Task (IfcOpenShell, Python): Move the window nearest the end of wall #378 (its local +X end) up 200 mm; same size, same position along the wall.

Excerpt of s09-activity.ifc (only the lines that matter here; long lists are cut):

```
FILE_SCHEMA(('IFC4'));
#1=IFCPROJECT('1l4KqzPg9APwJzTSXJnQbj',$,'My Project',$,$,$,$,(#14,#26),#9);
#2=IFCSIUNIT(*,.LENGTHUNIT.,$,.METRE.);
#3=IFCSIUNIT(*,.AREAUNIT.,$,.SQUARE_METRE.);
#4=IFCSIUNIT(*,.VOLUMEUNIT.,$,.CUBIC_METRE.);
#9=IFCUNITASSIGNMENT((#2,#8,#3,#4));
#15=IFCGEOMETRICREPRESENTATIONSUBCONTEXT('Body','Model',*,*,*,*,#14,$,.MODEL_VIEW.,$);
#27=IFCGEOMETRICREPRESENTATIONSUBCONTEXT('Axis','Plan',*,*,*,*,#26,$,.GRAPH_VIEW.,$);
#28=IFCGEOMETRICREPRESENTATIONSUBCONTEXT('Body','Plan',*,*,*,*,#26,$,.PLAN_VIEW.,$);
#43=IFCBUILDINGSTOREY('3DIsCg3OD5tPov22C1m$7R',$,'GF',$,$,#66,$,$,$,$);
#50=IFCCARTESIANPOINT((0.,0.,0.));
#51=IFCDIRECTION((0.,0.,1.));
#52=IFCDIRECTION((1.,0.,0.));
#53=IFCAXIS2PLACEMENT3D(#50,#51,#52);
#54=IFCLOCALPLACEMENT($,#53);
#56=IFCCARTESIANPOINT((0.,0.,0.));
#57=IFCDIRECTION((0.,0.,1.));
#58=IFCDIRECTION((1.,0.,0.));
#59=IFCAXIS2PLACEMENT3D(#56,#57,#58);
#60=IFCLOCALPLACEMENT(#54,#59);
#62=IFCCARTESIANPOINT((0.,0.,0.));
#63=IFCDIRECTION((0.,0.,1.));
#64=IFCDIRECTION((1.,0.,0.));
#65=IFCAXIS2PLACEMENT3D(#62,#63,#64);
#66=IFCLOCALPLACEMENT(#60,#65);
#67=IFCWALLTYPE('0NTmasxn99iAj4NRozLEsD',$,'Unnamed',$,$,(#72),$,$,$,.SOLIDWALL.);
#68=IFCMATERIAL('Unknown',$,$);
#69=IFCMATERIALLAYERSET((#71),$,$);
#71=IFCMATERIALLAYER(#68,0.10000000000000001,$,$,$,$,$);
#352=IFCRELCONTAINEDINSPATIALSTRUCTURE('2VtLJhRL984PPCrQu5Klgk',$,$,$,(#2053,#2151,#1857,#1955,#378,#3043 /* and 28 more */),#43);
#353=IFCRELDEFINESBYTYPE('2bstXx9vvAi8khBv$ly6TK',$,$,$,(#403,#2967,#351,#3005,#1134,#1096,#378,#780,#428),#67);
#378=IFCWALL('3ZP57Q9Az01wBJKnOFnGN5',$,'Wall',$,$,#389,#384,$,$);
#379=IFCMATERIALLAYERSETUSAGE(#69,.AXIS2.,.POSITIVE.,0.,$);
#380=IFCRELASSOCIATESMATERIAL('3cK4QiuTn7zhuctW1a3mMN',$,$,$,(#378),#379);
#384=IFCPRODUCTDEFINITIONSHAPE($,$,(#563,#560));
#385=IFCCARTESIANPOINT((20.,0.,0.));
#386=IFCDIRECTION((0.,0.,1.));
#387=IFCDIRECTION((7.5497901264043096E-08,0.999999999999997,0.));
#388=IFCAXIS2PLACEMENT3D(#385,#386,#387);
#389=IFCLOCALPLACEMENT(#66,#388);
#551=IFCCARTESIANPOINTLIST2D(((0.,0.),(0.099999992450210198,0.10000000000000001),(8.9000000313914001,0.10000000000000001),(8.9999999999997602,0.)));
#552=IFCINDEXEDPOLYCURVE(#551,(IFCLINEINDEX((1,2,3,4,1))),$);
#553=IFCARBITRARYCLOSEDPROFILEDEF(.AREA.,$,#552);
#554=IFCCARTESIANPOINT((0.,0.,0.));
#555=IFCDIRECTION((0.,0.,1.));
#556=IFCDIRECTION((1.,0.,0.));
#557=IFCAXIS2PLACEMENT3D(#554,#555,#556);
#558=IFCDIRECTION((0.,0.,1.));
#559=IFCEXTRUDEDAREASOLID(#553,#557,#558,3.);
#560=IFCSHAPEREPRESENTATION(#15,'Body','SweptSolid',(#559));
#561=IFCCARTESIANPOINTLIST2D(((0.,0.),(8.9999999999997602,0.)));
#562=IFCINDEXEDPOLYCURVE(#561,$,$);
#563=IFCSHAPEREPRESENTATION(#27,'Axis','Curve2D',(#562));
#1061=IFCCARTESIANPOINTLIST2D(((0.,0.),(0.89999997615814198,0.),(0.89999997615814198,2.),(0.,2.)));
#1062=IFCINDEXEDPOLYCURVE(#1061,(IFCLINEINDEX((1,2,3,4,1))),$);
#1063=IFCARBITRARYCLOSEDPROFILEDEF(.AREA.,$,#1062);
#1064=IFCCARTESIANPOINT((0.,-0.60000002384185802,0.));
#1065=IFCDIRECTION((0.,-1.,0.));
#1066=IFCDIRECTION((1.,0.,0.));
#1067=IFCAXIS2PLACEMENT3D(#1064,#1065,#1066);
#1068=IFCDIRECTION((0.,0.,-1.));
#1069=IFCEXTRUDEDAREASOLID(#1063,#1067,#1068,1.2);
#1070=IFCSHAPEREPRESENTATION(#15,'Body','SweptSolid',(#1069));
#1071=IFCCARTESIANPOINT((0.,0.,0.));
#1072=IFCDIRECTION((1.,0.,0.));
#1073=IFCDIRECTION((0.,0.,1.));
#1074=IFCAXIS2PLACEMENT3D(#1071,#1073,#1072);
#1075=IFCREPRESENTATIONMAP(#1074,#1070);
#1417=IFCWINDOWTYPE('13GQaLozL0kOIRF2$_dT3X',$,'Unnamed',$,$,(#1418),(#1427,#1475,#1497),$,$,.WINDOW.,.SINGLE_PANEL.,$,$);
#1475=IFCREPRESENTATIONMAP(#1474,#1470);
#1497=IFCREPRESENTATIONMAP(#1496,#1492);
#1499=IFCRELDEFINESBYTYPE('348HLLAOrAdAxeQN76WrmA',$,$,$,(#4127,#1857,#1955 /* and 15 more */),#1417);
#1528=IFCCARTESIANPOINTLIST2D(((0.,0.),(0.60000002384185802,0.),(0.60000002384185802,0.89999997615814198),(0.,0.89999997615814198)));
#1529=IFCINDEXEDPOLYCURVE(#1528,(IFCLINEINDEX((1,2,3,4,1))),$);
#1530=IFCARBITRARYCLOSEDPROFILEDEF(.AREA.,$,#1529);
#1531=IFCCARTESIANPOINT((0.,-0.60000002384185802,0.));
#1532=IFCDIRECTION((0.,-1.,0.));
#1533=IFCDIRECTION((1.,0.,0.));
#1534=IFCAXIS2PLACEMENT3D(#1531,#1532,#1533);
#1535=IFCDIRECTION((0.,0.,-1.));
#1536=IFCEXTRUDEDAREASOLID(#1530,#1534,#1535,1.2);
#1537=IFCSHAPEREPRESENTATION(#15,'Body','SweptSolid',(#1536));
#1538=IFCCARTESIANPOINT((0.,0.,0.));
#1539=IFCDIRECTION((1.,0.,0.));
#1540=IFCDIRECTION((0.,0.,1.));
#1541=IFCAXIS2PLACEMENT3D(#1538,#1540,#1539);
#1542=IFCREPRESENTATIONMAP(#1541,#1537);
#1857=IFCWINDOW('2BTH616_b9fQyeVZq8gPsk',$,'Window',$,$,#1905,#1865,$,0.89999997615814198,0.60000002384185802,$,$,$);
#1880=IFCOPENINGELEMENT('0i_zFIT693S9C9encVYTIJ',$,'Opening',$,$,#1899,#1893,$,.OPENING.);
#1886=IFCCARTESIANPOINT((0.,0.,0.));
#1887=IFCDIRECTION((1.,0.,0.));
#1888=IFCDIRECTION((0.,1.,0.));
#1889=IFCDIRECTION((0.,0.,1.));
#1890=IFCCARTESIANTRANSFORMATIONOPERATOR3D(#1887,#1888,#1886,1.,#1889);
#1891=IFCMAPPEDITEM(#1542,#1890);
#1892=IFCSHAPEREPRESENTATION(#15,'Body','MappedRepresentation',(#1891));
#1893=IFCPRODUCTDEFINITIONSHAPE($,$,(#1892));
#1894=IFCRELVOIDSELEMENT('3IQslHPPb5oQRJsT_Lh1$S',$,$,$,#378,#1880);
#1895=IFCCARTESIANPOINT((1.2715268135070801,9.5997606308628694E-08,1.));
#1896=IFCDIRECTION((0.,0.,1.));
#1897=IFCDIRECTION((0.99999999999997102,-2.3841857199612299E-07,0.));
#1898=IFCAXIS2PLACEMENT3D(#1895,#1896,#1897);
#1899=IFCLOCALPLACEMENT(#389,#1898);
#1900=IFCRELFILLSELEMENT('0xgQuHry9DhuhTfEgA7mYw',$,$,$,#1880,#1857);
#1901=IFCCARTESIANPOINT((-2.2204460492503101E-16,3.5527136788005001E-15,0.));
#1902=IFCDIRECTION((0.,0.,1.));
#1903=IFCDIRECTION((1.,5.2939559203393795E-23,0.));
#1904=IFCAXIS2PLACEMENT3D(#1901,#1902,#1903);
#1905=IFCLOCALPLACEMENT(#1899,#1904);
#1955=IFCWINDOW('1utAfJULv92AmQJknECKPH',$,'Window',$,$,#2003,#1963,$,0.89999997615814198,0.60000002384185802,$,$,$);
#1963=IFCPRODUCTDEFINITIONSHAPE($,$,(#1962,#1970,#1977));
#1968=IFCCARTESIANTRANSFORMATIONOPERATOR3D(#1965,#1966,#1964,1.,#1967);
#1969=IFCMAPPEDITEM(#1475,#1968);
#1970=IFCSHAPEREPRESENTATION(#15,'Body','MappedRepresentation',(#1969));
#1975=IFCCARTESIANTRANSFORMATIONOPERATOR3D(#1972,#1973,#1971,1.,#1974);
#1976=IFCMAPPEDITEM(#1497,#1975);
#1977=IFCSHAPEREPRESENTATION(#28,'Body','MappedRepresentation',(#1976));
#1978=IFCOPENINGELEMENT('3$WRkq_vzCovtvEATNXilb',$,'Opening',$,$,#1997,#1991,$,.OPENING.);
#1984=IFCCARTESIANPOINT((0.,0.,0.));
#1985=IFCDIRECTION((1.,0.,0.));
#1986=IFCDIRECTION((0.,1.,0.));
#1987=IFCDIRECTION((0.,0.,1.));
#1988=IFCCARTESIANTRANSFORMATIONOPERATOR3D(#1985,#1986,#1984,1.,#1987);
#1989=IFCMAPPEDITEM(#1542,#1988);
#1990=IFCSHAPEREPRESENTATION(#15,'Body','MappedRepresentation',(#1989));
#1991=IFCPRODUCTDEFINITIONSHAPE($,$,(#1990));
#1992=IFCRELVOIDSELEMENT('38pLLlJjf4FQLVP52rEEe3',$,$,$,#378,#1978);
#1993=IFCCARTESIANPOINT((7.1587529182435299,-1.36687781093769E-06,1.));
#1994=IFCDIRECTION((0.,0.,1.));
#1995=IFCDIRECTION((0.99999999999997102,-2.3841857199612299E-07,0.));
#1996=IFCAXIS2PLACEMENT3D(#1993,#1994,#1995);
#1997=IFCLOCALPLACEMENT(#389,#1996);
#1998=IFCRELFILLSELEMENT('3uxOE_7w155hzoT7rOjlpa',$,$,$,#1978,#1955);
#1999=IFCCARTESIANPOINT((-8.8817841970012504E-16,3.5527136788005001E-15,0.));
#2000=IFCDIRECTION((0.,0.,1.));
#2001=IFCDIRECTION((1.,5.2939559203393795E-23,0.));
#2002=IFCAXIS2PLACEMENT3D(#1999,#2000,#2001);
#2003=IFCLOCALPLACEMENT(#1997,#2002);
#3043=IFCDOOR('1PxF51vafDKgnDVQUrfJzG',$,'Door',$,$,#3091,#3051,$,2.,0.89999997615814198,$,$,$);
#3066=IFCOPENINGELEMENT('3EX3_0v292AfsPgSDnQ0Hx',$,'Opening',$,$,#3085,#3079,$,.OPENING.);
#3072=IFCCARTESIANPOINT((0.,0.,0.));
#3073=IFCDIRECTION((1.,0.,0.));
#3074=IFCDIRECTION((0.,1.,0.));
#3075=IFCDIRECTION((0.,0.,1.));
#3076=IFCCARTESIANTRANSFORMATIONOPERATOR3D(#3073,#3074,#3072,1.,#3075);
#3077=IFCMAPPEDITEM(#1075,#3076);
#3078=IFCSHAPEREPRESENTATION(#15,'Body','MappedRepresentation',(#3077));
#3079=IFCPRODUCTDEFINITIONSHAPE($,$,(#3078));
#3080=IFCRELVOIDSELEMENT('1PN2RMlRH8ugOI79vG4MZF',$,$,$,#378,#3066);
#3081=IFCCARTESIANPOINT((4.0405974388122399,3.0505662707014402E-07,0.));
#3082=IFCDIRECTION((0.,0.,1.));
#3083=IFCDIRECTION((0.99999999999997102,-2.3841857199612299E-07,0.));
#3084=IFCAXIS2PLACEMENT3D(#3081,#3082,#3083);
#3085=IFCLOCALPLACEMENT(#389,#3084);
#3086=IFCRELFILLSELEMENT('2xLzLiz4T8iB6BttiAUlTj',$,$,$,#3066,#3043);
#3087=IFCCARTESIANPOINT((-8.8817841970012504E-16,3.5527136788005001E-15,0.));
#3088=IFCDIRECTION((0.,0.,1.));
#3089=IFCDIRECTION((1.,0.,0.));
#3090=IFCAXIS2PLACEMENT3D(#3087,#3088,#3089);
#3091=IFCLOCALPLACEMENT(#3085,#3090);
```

```python
import numpy as np
import ifcopenshell
import ifcopenshell.api.geometry
import ifcopenshell.util.placement
import ifcopenshell.util.unit

model = ifcopenshell.open("s09-activity.ifc")
unit_scale = ifcopenshell.util.unit.calculate_unit_scale(model)

window = model.by_guid("1utAfJULv92AmQJknECKPH")
opening = window.FillsVoids[0].RelatingOpeningElement
dz = 0.2

shift = np.array([0.0, 0.0, dz])
# The window is placed relative to its opening, so it follows when the opening moves.
matrix = ifcopenshell.util.placement.get_local_placement(opening.ObjectPlacement)
matrix[:3, 3] += shift
ifcopenshell.api.geometry.edit_object_placement(
    model, product=opening, matrix=matrix, is_si=False, should_transform_children=True
)

print(f"moved by {dz * unit_scale:+.3f} m")

model.write("s09-activity_v2.ifc")
```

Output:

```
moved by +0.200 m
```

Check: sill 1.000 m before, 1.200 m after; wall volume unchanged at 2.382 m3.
